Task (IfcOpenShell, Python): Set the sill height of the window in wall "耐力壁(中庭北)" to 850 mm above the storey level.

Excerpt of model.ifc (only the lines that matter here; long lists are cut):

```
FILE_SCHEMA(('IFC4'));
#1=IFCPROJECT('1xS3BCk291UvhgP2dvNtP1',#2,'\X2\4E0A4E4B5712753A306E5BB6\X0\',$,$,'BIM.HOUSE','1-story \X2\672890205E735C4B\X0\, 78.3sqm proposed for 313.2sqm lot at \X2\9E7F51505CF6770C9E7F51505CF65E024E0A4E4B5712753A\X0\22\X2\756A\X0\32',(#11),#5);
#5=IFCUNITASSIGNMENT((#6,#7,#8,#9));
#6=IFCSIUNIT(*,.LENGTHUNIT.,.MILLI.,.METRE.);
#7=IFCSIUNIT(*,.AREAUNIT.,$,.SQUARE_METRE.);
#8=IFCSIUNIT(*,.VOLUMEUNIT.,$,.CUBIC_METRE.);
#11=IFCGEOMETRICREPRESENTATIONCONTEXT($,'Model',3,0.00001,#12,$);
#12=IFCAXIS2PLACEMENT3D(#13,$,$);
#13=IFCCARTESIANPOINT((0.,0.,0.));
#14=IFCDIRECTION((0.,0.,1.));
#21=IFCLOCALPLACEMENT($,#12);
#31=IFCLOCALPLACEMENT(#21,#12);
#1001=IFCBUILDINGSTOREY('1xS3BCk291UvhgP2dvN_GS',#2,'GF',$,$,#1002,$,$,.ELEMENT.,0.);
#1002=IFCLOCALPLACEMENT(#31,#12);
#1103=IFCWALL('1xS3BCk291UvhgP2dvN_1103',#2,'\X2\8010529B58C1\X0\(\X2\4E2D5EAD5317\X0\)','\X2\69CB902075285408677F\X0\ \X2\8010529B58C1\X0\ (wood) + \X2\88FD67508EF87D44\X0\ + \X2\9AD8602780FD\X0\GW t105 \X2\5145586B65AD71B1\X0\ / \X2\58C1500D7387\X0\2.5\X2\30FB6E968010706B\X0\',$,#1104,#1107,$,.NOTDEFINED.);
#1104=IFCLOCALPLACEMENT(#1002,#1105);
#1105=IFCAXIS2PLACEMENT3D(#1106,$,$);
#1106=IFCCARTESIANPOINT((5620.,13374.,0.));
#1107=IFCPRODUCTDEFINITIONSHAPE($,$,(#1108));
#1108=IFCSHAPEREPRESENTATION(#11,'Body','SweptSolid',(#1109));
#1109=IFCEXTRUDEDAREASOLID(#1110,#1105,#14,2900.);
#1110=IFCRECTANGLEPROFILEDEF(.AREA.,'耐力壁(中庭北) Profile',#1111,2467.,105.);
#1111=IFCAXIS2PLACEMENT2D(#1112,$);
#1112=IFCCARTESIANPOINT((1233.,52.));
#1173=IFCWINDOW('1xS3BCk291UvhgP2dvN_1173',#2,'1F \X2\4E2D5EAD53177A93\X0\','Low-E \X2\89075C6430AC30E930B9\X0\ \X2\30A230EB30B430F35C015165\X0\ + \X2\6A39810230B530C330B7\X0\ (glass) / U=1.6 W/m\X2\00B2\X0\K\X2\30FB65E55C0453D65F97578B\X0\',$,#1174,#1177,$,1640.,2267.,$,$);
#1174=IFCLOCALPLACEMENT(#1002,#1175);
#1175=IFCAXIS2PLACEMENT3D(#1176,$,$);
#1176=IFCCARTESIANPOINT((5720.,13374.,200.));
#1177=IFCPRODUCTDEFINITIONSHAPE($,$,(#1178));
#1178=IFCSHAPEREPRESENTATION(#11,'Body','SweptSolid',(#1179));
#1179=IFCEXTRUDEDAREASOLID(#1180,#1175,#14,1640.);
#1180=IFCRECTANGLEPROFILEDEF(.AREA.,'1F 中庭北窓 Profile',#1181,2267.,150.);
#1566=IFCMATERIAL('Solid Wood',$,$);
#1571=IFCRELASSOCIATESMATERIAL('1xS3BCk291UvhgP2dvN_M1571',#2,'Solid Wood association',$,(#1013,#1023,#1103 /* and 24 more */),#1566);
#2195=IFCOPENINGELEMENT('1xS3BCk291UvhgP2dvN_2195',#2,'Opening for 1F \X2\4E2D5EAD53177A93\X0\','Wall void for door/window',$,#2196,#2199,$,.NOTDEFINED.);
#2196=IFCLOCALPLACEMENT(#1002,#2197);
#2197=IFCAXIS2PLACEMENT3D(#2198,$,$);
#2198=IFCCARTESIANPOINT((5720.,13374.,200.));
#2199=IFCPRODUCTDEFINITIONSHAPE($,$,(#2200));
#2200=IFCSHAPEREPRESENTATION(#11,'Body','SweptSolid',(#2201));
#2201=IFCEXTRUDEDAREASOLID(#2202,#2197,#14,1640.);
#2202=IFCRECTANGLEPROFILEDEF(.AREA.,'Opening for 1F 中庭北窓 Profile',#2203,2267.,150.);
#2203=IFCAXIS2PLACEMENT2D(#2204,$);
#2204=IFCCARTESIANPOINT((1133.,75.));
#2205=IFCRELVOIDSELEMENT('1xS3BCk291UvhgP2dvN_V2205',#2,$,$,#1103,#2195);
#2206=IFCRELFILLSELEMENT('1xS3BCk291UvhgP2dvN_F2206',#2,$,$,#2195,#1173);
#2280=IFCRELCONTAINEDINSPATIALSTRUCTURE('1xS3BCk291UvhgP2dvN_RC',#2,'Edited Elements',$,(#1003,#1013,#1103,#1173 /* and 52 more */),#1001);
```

```python
import numpy as np
import ifcopenshell
import ifcopenshell.api.geometry
import ifcopenshell.geom
import ifcopenshell.util.element
import ifcopenshell.util.placement
import ifcopenshell.util.shape
import ifcopenshell.util.unit

model = ifcopenshell.open("model.ifc")
unit_scale = ifcopenshell.util.unit.calculate_unit_scale(model)

window = model.by_id(1173)
opening = window.FillsVoids[0].RelatingOpeningElement
storey = ifcopenshell.util.element.get_container(window, ifc_class="IfcBuildingStorey")
level = ifcopenshell.util.placement.get_local_placement(storey.ObjectPlacement)[2, 3]

# The opening's origin need not be at the sill, so measure its lowest point.
shape = ifcopenshell.geom.create_shape(ifcopenshell.geom.settings(), opening)
bottom = ifcopenshell.util.shape.get_shape_bottom_elevation(shape, shape.geometry) / unit_scale
dz = level + 0.85 / unit_scale - bottom

shift = np.array([0.0, 0.0, dz])
# The window is not placed relative to its opening, so move both.
for product in (opening, window):
    matrix = ifcopenshell.util.placement.get_local_placement(product.ObjectPlacement)
    matrix[:3, 3] += shift
    ifcopenshell.api.geometry.edit_object_placement(model, product=product, matrix=matrix, is_si=False)

print(f"moved by {dz * unit_scale:+.3f} m")

model.write("model-out.ifc")
```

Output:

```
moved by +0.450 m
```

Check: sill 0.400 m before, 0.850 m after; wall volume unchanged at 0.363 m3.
